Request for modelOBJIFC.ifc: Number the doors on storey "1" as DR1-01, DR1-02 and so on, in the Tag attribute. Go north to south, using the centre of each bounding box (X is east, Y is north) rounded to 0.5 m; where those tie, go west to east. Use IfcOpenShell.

First a look at what the model holds.

```python
import ifcopenshell
import ifcopenshell.util.element
import ifcopenshell.util.placement

model = ifcopenshell.open("modelOBJIFC.ifc")
print(model.schema)
storey = next(s for s in model.by_type("IfcBuildingStorey") if s.Name == "1")
doors = [e for e in ifcopenshell.util.element.get_decomposition(storey) if e.is_a("IfcDoor")]
for e in sorted(doors, key=lambda e: e.id()):
    origin = ifcopenshell.util.placement.get_local_placement(e.ObjectPlacement)[:3, 3]
    print(e.id(), e.Tag, e.Name, origin.round(2) + 0.0, sep=" | ")
```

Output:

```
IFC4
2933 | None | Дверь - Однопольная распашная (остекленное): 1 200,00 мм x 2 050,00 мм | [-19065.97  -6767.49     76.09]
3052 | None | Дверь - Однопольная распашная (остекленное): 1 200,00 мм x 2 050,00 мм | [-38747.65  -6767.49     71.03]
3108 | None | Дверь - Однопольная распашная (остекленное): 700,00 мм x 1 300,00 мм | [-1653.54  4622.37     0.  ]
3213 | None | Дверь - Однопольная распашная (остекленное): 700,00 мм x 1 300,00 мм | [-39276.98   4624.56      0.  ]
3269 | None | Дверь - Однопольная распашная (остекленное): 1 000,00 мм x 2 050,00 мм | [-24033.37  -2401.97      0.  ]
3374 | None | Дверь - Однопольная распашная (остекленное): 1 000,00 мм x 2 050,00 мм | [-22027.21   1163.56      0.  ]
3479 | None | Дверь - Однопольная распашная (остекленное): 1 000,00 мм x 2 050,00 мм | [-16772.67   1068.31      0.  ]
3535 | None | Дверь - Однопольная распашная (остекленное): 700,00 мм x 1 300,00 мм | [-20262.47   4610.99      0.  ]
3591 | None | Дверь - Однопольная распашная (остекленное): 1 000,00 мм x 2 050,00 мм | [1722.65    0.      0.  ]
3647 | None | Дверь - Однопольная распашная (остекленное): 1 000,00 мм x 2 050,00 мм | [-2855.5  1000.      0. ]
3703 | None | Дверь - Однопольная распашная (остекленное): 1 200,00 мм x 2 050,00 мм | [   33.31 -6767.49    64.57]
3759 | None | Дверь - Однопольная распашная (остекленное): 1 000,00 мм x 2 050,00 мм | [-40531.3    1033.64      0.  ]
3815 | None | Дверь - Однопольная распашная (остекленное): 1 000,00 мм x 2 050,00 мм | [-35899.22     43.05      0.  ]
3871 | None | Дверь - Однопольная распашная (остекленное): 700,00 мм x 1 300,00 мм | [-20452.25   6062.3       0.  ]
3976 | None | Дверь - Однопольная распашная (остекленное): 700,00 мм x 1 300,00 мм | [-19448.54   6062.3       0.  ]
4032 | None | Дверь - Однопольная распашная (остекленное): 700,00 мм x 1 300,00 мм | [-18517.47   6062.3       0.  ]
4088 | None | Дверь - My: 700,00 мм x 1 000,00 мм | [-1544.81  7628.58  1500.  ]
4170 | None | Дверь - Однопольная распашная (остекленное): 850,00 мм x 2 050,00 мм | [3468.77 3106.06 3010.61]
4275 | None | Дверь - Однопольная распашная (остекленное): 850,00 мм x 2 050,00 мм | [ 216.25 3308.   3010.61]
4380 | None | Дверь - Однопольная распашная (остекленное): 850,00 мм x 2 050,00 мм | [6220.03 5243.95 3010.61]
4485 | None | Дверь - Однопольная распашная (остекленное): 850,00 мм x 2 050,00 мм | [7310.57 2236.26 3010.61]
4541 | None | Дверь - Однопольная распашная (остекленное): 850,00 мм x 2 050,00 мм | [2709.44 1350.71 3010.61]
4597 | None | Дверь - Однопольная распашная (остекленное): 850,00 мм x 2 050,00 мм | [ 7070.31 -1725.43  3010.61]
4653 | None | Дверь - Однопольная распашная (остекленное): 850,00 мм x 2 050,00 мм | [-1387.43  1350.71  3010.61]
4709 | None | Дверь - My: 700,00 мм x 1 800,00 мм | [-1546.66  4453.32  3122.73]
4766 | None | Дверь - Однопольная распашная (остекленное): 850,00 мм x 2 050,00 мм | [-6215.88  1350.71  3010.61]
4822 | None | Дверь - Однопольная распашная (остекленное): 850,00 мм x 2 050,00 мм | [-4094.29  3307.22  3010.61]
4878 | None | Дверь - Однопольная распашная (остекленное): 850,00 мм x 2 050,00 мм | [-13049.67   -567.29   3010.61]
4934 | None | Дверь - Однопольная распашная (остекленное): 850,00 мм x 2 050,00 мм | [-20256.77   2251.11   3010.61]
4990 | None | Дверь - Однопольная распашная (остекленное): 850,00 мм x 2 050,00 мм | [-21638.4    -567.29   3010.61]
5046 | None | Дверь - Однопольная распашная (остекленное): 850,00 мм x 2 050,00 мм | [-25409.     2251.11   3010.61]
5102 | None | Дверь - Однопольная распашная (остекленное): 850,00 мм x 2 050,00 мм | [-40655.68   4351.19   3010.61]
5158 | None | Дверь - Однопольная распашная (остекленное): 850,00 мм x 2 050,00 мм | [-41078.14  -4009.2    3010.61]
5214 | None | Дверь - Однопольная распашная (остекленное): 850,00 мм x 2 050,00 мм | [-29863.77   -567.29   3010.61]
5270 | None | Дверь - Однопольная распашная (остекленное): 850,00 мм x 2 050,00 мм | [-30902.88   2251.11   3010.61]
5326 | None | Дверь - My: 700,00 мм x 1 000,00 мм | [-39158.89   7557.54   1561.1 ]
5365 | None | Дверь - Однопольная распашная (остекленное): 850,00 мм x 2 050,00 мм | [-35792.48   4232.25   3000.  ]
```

```python
import ifcopenshell
import ifcopenshell.geom
import ifcopenshell.util.element
import ifcopenshell.util.shape

model = ifcopenshell.open("modelOBJIFC.ifc")
settings = ifcopenshell.geom.settings()
settings.set("use-world-coords", True)


def centre(element):
    shape = ifcopenshell.geom.create_shape(settings, element)
    return ifcopenshell.util.shape.get_bbox_centroid(shape.geometry)


storey = next(s for s in model.by_type("IfcBuildingStorey") if s.Name == "1")
doors = [e for e in ifcopenshell.util.element.get_decomposition(storey) if e.is_a("IfcDoor")]

# Insertion points can sit at a corner or the storey origin, so sort by the geometry (in metres).
centres = {e: centre(e) for e in doors}
doors.sort(key=lambda e: (-round(centres[e][1] / 0.5), centres[e][0]))

for i, e in enumerate(doors, start=1):
    number = f"DR1-{i:02d}"
    e.Tag = number
    print(e.id(), number)

model.write("modelOBJIFC-out.ifc")
```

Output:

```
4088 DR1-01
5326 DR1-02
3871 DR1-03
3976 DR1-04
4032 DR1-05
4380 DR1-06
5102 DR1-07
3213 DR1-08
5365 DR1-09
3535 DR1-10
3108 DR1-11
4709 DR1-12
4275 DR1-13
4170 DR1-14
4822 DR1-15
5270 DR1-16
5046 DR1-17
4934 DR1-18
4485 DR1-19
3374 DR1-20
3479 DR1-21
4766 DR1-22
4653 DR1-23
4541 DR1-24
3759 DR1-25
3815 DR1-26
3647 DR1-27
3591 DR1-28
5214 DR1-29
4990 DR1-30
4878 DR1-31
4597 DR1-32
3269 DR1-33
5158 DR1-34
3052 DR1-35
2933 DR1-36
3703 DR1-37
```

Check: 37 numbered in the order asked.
